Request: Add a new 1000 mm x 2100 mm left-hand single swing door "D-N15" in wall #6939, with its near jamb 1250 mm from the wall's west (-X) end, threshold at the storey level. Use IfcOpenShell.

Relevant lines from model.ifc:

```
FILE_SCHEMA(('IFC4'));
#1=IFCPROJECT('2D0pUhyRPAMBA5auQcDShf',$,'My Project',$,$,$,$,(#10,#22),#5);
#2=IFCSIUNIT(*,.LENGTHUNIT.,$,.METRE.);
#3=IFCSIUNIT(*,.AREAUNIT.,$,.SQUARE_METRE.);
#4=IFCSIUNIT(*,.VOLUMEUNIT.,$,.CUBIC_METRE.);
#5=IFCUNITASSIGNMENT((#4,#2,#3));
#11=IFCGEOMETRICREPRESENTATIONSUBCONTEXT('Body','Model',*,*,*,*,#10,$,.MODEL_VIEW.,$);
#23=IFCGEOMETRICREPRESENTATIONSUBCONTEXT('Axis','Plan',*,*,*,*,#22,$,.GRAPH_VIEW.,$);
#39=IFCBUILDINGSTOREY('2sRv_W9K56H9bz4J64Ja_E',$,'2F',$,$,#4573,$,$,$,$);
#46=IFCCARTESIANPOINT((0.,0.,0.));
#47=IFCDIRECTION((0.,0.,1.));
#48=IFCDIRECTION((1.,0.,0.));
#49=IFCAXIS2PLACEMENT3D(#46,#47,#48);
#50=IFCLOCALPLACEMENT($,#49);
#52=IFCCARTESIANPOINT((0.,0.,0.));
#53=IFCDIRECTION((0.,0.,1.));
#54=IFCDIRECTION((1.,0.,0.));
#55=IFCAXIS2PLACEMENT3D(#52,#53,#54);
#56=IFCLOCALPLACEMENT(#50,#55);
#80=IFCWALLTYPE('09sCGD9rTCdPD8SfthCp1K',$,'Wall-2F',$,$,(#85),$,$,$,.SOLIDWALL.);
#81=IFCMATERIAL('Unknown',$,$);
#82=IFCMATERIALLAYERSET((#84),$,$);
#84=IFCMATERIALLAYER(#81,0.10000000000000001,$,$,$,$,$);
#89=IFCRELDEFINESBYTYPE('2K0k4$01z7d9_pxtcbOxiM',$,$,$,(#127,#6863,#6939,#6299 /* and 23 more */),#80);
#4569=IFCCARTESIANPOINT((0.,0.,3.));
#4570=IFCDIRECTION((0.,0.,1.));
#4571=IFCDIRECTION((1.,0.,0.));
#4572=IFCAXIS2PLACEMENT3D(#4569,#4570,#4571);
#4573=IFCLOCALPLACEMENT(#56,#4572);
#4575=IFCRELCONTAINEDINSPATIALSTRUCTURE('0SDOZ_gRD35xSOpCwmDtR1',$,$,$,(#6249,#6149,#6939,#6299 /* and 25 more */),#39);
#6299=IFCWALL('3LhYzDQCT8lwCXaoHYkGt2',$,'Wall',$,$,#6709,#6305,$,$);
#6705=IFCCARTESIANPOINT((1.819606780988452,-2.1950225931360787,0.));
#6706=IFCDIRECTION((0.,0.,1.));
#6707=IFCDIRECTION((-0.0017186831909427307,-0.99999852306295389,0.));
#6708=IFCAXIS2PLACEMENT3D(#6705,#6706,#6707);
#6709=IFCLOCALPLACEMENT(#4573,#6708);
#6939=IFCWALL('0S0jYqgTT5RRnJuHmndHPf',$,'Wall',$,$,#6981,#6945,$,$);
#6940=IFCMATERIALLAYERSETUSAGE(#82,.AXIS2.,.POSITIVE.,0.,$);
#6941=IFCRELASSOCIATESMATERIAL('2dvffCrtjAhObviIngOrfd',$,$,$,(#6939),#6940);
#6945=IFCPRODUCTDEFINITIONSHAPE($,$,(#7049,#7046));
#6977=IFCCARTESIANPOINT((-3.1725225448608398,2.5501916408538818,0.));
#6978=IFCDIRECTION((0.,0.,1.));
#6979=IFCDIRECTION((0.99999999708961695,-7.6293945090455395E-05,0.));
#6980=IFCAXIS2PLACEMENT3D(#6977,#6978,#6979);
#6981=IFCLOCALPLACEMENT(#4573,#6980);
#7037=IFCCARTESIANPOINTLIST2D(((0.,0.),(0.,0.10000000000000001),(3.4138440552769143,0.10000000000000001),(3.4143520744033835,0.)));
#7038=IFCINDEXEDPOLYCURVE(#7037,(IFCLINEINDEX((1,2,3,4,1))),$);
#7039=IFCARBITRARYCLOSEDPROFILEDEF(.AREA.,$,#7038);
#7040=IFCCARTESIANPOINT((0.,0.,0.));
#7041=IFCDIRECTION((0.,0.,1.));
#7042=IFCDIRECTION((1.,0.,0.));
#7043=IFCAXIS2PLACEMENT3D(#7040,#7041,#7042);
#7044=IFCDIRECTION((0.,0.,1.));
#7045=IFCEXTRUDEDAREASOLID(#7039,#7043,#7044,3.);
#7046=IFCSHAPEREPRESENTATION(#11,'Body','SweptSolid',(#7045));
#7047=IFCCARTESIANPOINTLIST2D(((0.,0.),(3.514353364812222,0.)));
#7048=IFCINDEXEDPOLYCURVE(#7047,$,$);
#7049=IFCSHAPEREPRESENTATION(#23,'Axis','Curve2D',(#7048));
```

```python
import numpy as np
import ifcopenshell
import ifcopenshell.api.feature
import ifcopenshell.api.geometry
import ifcopenshell.api.root
import ifcopenshell.api.spatial
import ifcopenshell.geom
import ifcopenshell.util.element
import ifcopenshell.util.placement
import ifcopenshell.util.representation
import ifcopenshell.util.shape
import ifcopenshell.util.unit

model = ifcopenshell.open("model.ifc")
unit_scale = ifcopenshell.util.unit.calculate_unit_scale(model)
settings = ifcopenshell.geom.settings()


def volume(element):
    """Net volume in cubic metres, openings subtracted."""
    shape = ifcopenshell.geom.create_shape(settings, element)
    return ifcopenshell.util.shape.get_volume(shape.geometry)


wall = model.by_guid("0S0jYqgTT5RRnJuHmndHPf")
storey = ifcopenshell.util.element.get_container(wall, ifc_class="IfcBuildingStorey")
context = ifcopenshell.util.representation.get_context(model, "Model", "Body", "MODEL_VIEW")
before = volume(wall)

width, height, from_end, sill = 1, 2.1, 1.25, 0.0  # metres

# The wall runs along its own X axis, and the end named is its -X end.
wall_shape = ifcopenshell.geom.create_shape(settings, wall)
x, y, z = ifcopenshell.util.shape.get_vertices(wall_shape.geometry).T
start = x.min() + from_end
face, thickness = float(y.min()), float(y.max() - y.min())
wall_matrix = ifcopenshell.util.placement.get_local_placement(wall.ObjectPlacement)
level = ifcopenshell.util.placement.get_local_placement(storey.ObjectPlacement)[2, 3]


def in_wall(x, y):
    """Placement at x, y metres in the wall's axes, at sill height."""
    matrix = wall_matrix.copy()
    matrix[:, 3] = wall_matrix @ np.array([x / unit_scale, y / unit_scale, 0.0, 1.0])
    matrix[2, 3] = level + sill / unit_scale
    return matrix


# Opening: a box that overshoots both wall faces by 50 mm.
opening = ifcopenshell.api.root.create_entity(model, ifc_class="IfcOpeningElement", predefined_type="OPENING")
box = ifcopenshell.api.geometry.add_wall_representation(
    model, context=context, length=width, height=height, thickness=thickness + 0.1
)
ifcopenshell.api.geometry.assign_representation(model, product=opening, representation=box)
ifcopenshell.api.geometry.edit_object_placement(model, product=opening, matrix=in_wall(start, face - 0.05), is_si=False)
ifcopenshell.api.feature.add_feature(model, feature=opening, element=wall)

door = ifcopenshell.api.root.create_entity(model, ifc_class="IfcDoor", name="D-N15", predefined_type="DOOR")
door.OverallWidth, door.OverallHeight = width / unit_scale, height / unit_scale
door.OperationType = "SINGLE_SWING_LEFT"
body = ifcopenshell.api.geometry.add_door_representation(
    model,
    context=context,
    overall_width=door.OverallWidth,
    overall_height=door.OverallHeight,
    operation_type="SINGLE_SWING_LEFT",
    lining_properties={"LiningDepth": thickness / unit_scale, "ThresholdDepth": thickness / unit_scale},
)
ifcopenshell.api.geometry.assign_representation(model, product=door, representation=body)
ifcopenshell.api.spatial.assign_container(model, products=[door], relating_structure=storey)
ifcopenshell.api.feature.add_filling(model, opening=opening, element=door)

# The lining spans the wall, so the door starts at the wall face.
ifcopenshell.api.geometry.edit_object_placement(model, product=door, matrix=in_wall(start, face), is_si=False)

after = volume(wall)

print(f"wall volume {before:.3f} -> {after:.3f} m3")

model.write("model_rev.ifc")
```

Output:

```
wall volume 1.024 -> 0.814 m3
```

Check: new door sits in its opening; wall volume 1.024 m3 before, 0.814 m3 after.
